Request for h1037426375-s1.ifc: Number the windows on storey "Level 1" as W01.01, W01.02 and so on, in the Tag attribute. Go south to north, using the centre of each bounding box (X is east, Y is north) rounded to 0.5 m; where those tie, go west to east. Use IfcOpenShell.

First a look at what the model holds.

```python
import ifcopenshell
import ifcopenshell.util.element
import ifcopenshell.util.placement

model = ifcopenshell.open("h1037426375-s1.ifc")
print(model.schema)
storey = next(s for s in model.by_type("IfcBuildingStorey") if s.Name == "Level 1")
windows = [e for e in ifcopenshell.util.element.get_decomposition(storey) if e.is_a("IfcWindow")]
for e in sorted(windows, key=lambda e: e.id()):
    origin = ifcopenshell.util.placement.get_local_placement(e.ObjectPlacement)[:3, 3]
    print(e.id(), e.Tag, e.Name, origin.round(2) + 0.0, sep=" | ")
```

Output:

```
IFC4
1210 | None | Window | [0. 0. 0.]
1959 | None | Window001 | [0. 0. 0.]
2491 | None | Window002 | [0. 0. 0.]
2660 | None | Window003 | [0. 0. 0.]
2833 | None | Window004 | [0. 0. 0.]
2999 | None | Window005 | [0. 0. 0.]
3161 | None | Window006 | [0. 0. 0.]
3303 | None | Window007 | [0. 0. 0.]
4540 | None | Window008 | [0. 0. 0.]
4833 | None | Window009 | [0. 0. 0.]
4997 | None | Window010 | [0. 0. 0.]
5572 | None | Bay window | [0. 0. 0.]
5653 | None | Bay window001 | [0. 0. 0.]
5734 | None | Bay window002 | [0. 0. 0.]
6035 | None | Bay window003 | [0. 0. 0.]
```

```python
import ifcopenshell
import ifcopenshell.geom
import ifcopenshell.util.element
import ifcopenshell.util.shape

model = ifcopenshell.open("h1037426375-s1.ifc")
settings = ifcopenshell.geom.settings()
settings.set("use-world-coords", True)


def centre(element):
    shape = ifcopenshell.geom.create_shape(settings, element)
    return ifcopenshell.util.shape.get_bbox_centroid(shape.geometry)


storey = next(s for s in model.by_type("IfcBuildingStorey") if s.Name == "Level 1")
windows = [e for e in ifcopenshell.util.element.get_decomposition(storey) if e.is_a("IfcWindow")]

# Insertion points can sit at a corner or the storey origin, so sort by the geometry (in metres).
centres = {e: centre(e) for e in windows}
windows.sort(key=lambda e: (round(centres[e][1] / 0.5), centres[e][0]))

for i, e in enumerate(windows, start=1):
    number = f"W01.{i:02d}"
    e.Tag = number
    print(e.id(), number)

model.write("h1037426375-s1_v2.ifc")
```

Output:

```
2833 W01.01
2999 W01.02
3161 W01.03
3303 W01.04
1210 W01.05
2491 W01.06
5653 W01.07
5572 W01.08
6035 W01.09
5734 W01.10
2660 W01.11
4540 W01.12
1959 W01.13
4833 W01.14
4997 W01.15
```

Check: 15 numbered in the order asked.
